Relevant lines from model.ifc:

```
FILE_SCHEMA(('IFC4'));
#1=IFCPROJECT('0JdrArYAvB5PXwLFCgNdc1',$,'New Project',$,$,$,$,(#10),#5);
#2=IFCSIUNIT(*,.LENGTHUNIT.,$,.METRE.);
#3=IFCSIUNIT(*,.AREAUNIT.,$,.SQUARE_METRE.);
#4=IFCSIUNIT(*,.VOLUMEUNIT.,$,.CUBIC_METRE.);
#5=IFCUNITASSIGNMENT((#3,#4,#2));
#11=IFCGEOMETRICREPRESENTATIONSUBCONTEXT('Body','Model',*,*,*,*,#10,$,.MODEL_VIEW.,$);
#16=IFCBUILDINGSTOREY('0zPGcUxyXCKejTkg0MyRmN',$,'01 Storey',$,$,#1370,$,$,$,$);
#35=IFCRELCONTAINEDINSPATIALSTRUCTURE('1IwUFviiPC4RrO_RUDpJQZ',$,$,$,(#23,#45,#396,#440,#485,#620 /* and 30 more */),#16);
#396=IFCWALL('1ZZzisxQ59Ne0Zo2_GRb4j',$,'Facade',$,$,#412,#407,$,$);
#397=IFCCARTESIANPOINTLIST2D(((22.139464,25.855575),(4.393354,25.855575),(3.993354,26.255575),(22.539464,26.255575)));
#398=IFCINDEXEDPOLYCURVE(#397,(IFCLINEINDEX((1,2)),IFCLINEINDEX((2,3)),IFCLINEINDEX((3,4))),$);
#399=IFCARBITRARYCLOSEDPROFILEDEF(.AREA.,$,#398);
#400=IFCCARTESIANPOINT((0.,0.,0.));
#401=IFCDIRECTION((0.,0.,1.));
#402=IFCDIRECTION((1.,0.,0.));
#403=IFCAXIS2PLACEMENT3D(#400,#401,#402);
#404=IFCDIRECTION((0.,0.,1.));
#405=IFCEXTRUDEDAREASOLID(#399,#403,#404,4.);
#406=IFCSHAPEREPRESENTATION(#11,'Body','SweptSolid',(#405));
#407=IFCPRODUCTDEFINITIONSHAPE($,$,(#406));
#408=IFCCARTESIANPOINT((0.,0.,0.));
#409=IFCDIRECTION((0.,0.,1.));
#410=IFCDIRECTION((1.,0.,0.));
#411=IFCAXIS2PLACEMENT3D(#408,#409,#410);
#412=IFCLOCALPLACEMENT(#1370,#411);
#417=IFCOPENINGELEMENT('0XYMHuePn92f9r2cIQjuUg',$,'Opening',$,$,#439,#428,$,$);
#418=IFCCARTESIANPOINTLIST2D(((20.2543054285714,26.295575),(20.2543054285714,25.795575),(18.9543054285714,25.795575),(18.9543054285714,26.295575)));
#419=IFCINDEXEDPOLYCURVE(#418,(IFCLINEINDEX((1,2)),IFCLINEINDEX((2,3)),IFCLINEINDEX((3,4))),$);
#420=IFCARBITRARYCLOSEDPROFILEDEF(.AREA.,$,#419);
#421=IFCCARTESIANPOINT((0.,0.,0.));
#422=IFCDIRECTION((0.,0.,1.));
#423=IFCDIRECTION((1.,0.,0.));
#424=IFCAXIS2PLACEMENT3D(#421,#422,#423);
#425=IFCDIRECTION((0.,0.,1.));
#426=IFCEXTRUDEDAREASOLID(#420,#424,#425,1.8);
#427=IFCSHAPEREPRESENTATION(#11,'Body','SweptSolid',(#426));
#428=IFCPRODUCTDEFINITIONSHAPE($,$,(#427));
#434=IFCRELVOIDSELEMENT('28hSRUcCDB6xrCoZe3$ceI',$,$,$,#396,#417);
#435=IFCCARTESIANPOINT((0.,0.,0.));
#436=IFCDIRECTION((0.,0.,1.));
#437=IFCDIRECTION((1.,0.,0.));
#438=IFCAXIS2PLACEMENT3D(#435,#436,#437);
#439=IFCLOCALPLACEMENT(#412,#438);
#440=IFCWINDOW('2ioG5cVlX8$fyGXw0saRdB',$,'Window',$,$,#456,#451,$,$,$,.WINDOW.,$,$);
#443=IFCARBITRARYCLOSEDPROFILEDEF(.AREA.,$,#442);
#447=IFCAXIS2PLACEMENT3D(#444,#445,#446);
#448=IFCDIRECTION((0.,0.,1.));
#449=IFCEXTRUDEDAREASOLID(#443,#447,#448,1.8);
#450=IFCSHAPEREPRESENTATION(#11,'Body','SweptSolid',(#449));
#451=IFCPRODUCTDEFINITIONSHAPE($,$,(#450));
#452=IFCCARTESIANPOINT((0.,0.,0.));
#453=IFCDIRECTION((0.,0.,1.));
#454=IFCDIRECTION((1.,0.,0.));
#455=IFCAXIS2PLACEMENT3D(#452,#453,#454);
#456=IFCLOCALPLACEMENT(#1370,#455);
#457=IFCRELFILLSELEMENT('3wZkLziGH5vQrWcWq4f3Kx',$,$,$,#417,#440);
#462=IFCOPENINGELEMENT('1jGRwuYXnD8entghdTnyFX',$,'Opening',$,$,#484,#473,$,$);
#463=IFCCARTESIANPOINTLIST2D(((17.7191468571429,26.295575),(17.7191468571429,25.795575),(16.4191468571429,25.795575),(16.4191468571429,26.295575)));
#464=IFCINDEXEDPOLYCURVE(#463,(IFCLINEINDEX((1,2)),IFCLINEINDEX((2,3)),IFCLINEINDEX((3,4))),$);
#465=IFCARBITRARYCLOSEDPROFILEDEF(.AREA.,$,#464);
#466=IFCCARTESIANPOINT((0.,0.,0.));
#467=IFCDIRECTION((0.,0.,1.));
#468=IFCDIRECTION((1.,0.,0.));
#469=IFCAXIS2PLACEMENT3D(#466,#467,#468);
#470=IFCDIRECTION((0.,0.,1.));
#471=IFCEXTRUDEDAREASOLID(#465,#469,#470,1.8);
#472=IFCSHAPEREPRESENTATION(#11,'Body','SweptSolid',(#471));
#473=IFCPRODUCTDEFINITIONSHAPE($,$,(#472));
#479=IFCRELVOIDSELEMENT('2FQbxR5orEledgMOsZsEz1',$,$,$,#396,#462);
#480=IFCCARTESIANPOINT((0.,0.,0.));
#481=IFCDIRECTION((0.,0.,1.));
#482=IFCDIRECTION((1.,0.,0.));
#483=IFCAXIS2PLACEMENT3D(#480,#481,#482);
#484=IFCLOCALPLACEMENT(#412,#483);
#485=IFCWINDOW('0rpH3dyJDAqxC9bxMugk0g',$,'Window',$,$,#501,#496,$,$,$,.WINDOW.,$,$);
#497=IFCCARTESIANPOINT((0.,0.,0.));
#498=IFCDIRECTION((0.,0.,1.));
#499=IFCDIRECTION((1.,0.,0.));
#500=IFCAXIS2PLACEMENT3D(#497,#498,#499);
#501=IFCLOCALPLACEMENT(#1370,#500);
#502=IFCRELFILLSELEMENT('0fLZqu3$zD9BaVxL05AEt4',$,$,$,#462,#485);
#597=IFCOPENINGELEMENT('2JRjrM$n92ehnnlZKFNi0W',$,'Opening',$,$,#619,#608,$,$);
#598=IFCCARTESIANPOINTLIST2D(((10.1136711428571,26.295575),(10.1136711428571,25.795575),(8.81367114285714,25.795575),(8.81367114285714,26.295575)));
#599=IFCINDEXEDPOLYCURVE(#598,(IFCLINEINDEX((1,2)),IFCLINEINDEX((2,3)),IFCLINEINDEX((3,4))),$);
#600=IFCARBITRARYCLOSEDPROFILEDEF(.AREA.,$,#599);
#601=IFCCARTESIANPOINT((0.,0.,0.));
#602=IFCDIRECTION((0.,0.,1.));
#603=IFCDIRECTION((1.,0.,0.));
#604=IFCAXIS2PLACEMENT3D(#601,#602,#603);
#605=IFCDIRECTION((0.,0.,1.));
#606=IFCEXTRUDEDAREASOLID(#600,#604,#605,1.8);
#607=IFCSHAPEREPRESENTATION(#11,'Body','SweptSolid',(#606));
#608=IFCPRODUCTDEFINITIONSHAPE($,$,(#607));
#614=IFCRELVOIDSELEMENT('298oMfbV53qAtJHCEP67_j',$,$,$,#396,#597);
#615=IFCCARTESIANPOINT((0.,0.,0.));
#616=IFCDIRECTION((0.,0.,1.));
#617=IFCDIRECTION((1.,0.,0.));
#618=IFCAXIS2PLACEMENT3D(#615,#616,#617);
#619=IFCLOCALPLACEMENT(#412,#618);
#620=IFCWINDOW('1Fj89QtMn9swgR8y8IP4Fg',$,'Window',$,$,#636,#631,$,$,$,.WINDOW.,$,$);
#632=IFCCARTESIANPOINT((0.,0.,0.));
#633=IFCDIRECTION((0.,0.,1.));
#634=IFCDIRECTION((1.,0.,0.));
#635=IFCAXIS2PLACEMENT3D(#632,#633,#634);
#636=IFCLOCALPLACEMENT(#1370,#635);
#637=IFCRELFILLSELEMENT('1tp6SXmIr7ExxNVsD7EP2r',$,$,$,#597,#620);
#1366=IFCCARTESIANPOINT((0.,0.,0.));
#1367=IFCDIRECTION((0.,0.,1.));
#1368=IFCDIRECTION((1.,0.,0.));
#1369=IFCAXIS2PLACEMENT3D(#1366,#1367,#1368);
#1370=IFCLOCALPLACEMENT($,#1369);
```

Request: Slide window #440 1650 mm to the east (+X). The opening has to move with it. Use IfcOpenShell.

```python
import ifcopenshell
import ifcopenshell.api.geometry
import ifcopenshell.util.placement
import ifcopenshell.util.unit

model = ifcopenshell.open("model.ifc")
unit_scale = ifcopenshell.util.unit.calculate_unit_scale(model)

window = model.by_guid("2ioG5cVlX8$fyGXw0saRdB")
opening = window.FillsVoids[0].RelatingOpeningElement
wall = opening.VoidsElements[0].RelatingBuildingElement

wall_matrix = ifcopenshell.util.placement.get_local_placement(wall.ObjectPlacement)
shift = wall_matrix[:3, 0] * 1.65 / unit_scale
before = ifcopenshell.util.placement.get_local_placement(window.ObjectPlacement)[:3, 3].copy()

# The window is not placed relative to its opening, so move both.
for product in (opening, window):
    matrix = ifcopenshell.util.placement.get_local_placement(product.ObjectPlacement)
    matrix[:3, 3] += shift
    ifcopenshell.api.geometry.edit_object_placement(model, product=product, matrix=matrix, is_si=False)

after = ifcopenshell.util.placement.get_local_placement(window.ObjectPlacement)[:3, 3]
print("window moved by", (after - before).round(3) + 0.0)

model.write("model_updated.ifc")
```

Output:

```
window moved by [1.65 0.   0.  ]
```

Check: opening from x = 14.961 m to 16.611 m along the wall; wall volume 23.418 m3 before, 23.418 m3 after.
